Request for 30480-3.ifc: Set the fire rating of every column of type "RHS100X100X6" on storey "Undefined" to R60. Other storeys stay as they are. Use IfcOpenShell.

First a look at what the model holds.

```python
import ifcopenshell
import ifcopenshell.util.element

model = ifcopenshell.open("30480-3.ifc")
print(model.schema)
storey = next(s for s in model.by_type("IfcBuildingStorey") if s.Name == "Undefined")
columns = [e for e in ifcopenshell.util.element.get_decomposition(storey) if e.is_a("IfcColumn")]
seen = {}
for e in columns:
    element_type = ifcopenshell.util.element.get_type(e)
    key = (element_type.Name if element_type != e and element_type else None, ifcopenshell.util.element.get_pset(e, "Pset_ColumnCommon", "FireRating"))
    seen[key] = seen.get(key, 0) + 1
for (name, value), count in sorted(seen.items(), key=str):
    print(count, "x", name, "|", value)
```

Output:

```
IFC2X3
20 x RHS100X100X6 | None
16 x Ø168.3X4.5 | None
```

```python
import ifcopenshell
import ifcopenshell.api.pset
import ifcopenshell.util.element

model = ifcopenshell.open("30480-3.ifc")

storey = next(s for s in model.by_type("IfcBuildingStorey") if s.Name == "Undefined")
columns = [e for e in ifcopenshell.util.element.get_decomposition(storey) if e.is_a("IfcColumn")]

count = 0
for e in columns:
    element_type = ifcopenshell.util.element.get_type(e)
    if element_type in (None, e) or element_type.Name != "RHS100X100X6":
        continue
    found = ifcopenshell.util.element.get_pset(e, "Pset_ColumnCommon", should_inherit=False)
    if found:
        pset = model.by_id(found["id"])
        if len(ifcopenshell.util.element.get_elements_by_pset(pset)) > 1:
            pset = ifcopenshell.api.pset.unshare_pset(model, products=[e], pset=pset)[0]
    else:
        pset = ifcopenshell.api.pset.add_pset(model, product=e, name="Pset_ColumnCommon")
    ifcopenshell.api.pset.edit_pset(model, pset=pset, properties={"FireRating": "R60"})
    count += 1

print(count, "columns updated")

model.write("30480-3_rev.ifc")
```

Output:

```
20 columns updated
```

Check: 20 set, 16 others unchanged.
